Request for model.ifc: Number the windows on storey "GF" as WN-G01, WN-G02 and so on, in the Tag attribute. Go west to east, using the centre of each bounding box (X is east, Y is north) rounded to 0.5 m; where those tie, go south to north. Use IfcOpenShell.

First a look at what the model holds.

```python
import ifcopenshell
import ifcopenshell.util.element
import ifcopenshell.util.placement

model = ifcopenshell.open("model.ifc")
print(model.schema)
storey = next(s for s in model.by_type("IfcBuildingStorey") if s.Name == "GF")
windows = [e for e in ifcopenshell.util.element.get_decomposition(storey) if e.is_a("IfcWindow")]
for e in sorted(windows, key=lambda e: e.id()):
    origin = ifcopenshell.util.placement.get_local_placement(e.ObjectPlacement)[:3, 3]
    print(e.id(), e.Tag, e.Name, origin.round(2) + 0.0, sep=" | ")
```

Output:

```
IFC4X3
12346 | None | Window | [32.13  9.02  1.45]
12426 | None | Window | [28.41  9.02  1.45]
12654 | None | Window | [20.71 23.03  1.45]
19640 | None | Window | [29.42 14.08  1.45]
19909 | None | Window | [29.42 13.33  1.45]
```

```python
import ifcopenshell
import ifcopenshell.geom
import ifcopenshell.util.element
import ifcopenshell.util.shape

model = ifcopenshell.open("model.ifc")
settings = ifcopenshell.geom.settings()
settings.set("use-world-coords", True)


def centre(element):
    shape = ifcopenshell.geom.create_shape(settings, element)
    return ifcopenshell.util.shape.get_bbox_centroid(shape.geometry)


storey = next(s for s in model.by_type("IfcBuildingStorey") if s.Name == "GF")
windows = [e for e in ifcopenshell.util.element.get_decomposition(storey) if e.is_a("IfcWindow")]

# Insertion points can sit at a corner or the storey origin, so sort by the geometry (in metres).
centres = {e: centre(e) for e in windows}
windows.sort(key=lambda e: (round(centres[e][0] / 0.5), centres[e][1]))

for i, e in enumerate(windows, start=1):
    number = f"WN-G{i:02d}"
    e.Tag = number
    print(e.id(), number)

model.write("model_v2.ifc")
```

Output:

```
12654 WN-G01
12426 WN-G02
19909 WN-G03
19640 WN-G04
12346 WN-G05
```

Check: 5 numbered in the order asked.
